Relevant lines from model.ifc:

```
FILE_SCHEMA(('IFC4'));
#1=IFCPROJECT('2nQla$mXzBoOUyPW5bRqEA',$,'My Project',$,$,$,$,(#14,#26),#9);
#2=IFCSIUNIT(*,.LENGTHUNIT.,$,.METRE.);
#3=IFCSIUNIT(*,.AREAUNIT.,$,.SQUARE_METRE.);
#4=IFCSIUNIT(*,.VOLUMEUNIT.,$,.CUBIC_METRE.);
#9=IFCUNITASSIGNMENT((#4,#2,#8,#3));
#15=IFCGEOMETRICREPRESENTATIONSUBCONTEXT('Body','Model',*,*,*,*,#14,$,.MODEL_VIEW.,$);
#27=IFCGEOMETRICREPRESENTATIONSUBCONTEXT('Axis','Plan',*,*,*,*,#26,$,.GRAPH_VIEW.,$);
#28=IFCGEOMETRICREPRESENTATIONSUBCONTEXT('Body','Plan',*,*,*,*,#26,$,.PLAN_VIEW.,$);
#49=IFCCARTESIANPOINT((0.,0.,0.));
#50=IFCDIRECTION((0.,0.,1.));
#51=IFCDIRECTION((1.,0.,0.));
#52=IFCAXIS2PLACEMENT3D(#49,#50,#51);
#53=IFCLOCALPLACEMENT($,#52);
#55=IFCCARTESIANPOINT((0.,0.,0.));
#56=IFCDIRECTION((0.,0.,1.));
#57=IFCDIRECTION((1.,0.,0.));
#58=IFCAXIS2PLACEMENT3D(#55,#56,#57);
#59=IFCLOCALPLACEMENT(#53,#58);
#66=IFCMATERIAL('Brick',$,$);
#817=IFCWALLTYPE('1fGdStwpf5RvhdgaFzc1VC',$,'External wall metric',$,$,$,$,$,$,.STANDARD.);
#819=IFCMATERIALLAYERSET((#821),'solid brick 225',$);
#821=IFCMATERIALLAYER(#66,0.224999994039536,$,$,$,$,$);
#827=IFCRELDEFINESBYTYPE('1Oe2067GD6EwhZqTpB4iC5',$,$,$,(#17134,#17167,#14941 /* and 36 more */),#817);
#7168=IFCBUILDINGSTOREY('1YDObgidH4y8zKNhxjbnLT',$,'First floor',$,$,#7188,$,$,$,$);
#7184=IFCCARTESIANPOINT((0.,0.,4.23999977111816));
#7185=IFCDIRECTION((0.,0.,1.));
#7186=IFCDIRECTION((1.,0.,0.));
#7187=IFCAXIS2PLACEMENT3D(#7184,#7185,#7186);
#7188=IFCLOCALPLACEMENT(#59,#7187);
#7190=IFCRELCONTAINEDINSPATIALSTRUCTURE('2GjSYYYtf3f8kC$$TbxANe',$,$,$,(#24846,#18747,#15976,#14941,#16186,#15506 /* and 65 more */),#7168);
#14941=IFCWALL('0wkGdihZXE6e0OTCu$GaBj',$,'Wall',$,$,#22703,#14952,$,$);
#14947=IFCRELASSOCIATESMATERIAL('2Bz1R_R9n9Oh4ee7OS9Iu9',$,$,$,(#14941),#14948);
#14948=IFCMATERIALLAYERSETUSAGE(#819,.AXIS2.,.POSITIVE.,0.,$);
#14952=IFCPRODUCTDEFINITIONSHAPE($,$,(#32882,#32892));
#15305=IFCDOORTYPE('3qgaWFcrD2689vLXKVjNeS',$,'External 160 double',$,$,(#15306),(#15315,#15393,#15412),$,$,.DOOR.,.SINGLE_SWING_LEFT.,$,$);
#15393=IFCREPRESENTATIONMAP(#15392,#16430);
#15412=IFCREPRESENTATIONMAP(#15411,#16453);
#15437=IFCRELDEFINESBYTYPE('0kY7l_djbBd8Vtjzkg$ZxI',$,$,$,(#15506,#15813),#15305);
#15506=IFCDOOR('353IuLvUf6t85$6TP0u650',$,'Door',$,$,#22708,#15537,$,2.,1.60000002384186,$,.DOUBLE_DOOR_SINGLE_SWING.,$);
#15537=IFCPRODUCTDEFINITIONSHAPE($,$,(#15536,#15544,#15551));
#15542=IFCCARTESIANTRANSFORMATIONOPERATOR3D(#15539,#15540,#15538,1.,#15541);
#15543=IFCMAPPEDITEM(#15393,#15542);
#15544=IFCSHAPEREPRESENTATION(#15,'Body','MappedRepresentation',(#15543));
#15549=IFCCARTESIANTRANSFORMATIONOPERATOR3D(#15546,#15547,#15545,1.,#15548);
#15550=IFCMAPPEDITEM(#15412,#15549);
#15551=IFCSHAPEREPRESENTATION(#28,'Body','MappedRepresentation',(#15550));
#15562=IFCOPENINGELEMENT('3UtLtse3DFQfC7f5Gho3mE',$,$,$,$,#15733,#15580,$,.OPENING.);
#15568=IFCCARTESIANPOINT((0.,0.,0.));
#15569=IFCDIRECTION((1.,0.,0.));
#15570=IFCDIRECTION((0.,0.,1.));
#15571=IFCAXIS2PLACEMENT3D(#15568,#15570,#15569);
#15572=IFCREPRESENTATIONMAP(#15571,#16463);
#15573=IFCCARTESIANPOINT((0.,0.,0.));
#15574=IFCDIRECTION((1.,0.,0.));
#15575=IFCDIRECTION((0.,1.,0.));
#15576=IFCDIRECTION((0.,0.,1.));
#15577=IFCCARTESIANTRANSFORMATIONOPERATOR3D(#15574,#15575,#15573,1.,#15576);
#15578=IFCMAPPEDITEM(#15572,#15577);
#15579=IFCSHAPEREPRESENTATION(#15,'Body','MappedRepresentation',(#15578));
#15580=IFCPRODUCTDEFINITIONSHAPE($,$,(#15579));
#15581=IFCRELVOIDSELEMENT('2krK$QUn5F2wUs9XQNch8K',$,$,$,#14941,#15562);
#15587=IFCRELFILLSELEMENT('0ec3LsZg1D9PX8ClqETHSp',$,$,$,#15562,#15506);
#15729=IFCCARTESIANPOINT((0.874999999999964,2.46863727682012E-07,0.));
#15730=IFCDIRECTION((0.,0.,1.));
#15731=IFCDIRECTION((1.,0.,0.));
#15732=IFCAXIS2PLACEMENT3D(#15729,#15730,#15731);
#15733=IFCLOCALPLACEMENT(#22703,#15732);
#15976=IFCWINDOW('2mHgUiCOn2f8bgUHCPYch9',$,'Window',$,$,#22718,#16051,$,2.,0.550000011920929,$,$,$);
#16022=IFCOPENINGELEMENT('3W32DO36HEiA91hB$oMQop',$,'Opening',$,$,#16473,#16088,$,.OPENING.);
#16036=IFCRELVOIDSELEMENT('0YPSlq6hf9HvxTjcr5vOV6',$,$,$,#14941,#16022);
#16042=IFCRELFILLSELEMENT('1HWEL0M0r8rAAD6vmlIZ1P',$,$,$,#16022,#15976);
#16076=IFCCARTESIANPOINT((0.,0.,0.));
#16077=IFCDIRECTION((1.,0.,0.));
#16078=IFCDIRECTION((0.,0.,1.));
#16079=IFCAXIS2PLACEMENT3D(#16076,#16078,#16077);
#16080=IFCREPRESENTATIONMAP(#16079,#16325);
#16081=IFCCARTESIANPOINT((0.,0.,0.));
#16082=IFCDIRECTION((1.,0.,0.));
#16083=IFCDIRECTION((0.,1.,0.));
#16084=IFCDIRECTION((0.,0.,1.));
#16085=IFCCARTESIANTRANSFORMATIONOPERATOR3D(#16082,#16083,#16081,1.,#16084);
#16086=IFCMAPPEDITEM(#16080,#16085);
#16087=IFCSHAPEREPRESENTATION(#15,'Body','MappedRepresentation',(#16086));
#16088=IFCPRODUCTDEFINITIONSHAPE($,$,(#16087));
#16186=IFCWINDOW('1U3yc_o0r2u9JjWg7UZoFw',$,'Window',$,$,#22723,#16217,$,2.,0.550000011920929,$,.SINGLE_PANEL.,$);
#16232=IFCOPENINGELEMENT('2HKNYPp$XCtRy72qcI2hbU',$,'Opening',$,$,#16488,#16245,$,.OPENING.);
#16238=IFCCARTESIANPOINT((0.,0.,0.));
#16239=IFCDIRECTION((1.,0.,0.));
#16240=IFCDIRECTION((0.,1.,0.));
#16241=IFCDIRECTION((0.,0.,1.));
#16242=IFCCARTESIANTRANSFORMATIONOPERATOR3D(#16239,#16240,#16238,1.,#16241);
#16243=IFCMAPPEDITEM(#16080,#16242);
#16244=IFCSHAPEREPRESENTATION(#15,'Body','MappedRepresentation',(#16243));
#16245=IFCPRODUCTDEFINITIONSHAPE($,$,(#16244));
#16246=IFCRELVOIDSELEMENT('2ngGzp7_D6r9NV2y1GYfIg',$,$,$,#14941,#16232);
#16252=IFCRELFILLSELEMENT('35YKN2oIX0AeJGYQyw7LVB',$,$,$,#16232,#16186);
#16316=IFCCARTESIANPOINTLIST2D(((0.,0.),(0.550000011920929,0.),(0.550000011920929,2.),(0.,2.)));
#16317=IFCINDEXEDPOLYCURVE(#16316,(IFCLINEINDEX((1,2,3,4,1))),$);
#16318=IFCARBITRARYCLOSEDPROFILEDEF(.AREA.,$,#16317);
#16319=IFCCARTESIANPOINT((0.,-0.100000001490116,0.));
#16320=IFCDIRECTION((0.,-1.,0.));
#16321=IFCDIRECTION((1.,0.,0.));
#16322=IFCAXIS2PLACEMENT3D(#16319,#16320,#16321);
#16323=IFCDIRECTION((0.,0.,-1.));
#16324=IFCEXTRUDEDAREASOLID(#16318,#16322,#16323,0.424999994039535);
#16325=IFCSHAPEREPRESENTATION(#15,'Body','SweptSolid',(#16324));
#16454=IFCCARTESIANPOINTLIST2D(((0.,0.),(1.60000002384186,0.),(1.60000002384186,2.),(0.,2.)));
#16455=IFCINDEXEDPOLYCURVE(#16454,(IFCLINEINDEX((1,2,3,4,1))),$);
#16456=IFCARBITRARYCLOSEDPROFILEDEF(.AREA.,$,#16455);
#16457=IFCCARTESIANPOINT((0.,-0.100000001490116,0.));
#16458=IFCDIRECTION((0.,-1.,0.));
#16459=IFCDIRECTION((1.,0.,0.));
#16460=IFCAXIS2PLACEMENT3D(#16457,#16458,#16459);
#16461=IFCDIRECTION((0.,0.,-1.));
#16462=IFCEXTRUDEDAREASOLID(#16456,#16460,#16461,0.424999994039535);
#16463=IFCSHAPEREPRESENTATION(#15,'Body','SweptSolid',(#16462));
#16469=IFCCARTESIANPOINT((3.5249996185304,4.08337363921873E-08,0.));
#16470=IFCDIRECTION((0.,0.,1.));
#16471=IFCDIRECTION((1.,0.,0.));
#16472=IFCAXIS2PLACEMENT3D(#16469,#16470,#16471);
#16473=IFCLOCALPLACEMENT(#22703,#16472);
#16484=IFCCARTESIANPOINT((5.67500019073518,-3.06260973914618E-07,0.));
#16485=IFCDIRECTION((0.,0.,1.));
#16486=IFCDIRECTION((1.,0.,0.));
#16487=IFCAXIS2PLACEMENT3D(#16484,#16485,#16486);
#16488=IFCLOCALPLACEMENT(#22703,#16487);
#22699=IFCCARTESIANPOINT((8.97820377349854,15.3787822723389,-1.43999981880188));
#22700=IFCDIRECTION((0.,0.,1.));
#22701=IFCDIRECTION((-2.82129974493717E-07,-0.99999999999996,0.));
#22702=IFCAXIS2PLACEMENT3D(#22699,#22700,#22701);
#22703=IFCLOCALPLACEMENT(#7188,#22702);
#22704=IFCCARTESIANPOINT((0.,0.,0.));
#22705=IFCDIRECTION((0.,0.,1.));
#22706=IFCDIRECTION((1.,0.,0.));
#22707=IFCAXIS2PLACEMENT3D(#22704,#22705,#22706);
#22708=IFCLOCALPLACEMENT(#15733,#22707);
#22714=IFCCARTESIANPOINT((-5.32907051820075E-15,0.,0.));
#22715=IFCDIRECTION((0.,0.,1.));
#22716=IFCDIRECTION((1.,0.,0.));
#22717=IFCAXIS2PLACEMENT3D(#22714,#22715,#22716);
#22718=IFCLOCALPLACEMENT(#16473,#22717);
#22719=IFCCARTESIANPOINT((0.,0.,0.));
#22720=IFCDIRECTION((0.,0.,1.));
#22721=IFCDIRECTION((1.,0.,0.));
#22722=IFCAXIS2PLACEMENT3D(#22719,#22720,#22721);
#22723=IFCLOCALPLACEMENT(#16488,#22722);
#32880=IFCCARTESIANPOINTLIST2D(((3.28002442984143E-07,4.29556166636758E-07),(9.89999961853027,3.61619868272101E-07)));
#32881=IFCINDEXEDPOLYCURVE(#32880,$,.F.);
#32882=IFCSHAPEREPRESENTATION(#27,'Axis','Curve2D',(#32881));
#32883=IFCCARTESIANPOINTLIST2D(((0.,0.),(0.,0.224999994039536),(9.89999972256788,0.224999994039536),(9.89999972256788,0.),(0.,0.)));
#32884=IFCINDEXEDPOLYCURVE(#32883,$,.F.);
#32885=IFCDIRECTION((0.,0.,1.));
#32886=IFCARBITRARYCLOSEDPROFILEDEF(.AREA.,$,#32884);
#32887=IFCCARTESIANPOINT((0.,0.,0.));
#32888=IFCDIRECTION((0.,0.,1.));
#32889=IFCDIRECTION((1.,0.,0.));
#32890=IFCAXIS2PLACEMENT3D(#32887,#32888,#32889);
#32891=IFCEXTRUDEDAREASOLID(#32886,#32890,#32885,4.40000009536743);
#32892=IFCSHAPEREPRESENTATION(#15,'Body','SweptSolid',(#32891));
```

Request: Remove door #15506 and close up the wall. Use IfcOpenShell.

```python
import ifcopenshell
import ifcopenshell.api.feature
import ifcopenshell.api.root
import ifcopenshell.geom
import ifcopenshell.util.shape

model = ifcopenshell.open("model.ifc")
settings = ifcopenshell.geom.settings()


def volume(element):
    """Net volume in cubic metres, openings subtracted."""
    shape = ifcopenshell.geom.create_shape(settings, element)
    return ifcopenshell.util.shape.get_volume(shape.geometry)


door = model.by_guid("353IuLvUf6t85$6TP0u650")
opening = door.FillsVoids[0].RelatingOpeningElement
wall = opening.VoidsElements[0].RelatingBuildingElement
before = volume(wall)

ifcopenshell.api.root.remove_product(model, product=door)
ifcopenshell.api.feature.remove_feature(model, feature=opening)

after = volume(wall)

print(f"wall volume {before:.3f} -> {after:.3f} m3")

model.write("model_v2.ifc")
```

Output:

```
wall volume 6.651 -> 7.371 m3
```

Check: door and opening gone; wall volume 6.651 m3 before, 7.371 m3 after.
